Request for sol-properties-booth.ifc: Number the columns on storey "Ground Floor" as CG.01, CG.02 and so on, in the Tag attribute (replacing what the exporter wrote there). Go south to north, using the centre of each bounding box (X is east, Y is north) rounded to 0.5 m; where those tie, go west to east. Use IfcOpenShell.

First a look at what the model holds.

```python
import ifcopenshell
import ifcopenshell.util.element
import ifcopenshell.util.placement

model = ifcopenshell.open("sol-properties-booth.ifc")
print(model.schema)
storey = next(s for s in model.by_type("IfcBuildingStorey") if s.Name == "Ground Floor")
columns = [e for e in ifcopenshell.util.element.get_decomposition(storey) if e.is_a("IfcColumn")]
for e in sorted(columns, key=lambda e: e.id()):
    origin = ifcopenshell.util.placement.get_local_placement(e.ObjectPlacement)[:3, 3]
    print(e.id(), e.Tag, e.Name, origin.round(2) + 0.0, sep=" | ")
```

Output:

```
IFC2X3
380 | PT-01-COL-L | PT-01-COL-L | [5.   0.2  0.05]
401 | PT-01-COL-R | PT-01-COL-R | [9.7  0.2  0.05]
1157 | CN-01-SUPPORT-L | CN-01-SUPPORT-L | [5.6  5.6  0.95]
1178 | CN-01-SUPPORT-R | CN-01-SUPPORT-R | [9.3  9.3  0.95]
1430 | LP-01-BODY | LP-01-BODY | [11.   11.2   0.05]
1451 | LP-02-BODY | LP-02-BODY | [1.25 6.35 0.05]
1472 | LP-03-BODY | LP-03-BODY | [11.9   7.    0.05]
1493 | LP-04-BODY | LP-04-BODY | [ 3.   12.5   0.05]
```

```python
import ifcopenshell
import ifcopenshell.geom
import ifcopenshell.util.element
import ifcopenshell.util.shape

model = ifcopenshell.open("sol-properties-booth.ifc")
settings = ifcopenshell.geom.settings()
settings.set("use-world-coords", True)


def centre(element):
    shape = ifcopenshell.geom.create_shape(settings, element)
    return ifcopenshell.util.shape.get_bbox_centroid(shape.geometry)


storey = next(s for s in model.by_type("IfcBuildingStorey") if s.Name == "Ground Floor")
columns = [e for e in ifcopenshell.util.element.get_decomposition(storey) if e.is_a("IfcColumn")]

# Insertion points can sit at a corner or the storey origin, so sort by the geometry (in metres).
centres = {e: centre(e) for e in columns}
columns.sort(key=lambda e: (round(centres[e][1] / 0.5), centres[e][0]))

for i, e in enumerate(columns, start=1):
    number = f"CG.{i:02d}"
    e.Tag = number
    print(e.id(), number)

model.write("sol-properties-booth_v2.ifc")
```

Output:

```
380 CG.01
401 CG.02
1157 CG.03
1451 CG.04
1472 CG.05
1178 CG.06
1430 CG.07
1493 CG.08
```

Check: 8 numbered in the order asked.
